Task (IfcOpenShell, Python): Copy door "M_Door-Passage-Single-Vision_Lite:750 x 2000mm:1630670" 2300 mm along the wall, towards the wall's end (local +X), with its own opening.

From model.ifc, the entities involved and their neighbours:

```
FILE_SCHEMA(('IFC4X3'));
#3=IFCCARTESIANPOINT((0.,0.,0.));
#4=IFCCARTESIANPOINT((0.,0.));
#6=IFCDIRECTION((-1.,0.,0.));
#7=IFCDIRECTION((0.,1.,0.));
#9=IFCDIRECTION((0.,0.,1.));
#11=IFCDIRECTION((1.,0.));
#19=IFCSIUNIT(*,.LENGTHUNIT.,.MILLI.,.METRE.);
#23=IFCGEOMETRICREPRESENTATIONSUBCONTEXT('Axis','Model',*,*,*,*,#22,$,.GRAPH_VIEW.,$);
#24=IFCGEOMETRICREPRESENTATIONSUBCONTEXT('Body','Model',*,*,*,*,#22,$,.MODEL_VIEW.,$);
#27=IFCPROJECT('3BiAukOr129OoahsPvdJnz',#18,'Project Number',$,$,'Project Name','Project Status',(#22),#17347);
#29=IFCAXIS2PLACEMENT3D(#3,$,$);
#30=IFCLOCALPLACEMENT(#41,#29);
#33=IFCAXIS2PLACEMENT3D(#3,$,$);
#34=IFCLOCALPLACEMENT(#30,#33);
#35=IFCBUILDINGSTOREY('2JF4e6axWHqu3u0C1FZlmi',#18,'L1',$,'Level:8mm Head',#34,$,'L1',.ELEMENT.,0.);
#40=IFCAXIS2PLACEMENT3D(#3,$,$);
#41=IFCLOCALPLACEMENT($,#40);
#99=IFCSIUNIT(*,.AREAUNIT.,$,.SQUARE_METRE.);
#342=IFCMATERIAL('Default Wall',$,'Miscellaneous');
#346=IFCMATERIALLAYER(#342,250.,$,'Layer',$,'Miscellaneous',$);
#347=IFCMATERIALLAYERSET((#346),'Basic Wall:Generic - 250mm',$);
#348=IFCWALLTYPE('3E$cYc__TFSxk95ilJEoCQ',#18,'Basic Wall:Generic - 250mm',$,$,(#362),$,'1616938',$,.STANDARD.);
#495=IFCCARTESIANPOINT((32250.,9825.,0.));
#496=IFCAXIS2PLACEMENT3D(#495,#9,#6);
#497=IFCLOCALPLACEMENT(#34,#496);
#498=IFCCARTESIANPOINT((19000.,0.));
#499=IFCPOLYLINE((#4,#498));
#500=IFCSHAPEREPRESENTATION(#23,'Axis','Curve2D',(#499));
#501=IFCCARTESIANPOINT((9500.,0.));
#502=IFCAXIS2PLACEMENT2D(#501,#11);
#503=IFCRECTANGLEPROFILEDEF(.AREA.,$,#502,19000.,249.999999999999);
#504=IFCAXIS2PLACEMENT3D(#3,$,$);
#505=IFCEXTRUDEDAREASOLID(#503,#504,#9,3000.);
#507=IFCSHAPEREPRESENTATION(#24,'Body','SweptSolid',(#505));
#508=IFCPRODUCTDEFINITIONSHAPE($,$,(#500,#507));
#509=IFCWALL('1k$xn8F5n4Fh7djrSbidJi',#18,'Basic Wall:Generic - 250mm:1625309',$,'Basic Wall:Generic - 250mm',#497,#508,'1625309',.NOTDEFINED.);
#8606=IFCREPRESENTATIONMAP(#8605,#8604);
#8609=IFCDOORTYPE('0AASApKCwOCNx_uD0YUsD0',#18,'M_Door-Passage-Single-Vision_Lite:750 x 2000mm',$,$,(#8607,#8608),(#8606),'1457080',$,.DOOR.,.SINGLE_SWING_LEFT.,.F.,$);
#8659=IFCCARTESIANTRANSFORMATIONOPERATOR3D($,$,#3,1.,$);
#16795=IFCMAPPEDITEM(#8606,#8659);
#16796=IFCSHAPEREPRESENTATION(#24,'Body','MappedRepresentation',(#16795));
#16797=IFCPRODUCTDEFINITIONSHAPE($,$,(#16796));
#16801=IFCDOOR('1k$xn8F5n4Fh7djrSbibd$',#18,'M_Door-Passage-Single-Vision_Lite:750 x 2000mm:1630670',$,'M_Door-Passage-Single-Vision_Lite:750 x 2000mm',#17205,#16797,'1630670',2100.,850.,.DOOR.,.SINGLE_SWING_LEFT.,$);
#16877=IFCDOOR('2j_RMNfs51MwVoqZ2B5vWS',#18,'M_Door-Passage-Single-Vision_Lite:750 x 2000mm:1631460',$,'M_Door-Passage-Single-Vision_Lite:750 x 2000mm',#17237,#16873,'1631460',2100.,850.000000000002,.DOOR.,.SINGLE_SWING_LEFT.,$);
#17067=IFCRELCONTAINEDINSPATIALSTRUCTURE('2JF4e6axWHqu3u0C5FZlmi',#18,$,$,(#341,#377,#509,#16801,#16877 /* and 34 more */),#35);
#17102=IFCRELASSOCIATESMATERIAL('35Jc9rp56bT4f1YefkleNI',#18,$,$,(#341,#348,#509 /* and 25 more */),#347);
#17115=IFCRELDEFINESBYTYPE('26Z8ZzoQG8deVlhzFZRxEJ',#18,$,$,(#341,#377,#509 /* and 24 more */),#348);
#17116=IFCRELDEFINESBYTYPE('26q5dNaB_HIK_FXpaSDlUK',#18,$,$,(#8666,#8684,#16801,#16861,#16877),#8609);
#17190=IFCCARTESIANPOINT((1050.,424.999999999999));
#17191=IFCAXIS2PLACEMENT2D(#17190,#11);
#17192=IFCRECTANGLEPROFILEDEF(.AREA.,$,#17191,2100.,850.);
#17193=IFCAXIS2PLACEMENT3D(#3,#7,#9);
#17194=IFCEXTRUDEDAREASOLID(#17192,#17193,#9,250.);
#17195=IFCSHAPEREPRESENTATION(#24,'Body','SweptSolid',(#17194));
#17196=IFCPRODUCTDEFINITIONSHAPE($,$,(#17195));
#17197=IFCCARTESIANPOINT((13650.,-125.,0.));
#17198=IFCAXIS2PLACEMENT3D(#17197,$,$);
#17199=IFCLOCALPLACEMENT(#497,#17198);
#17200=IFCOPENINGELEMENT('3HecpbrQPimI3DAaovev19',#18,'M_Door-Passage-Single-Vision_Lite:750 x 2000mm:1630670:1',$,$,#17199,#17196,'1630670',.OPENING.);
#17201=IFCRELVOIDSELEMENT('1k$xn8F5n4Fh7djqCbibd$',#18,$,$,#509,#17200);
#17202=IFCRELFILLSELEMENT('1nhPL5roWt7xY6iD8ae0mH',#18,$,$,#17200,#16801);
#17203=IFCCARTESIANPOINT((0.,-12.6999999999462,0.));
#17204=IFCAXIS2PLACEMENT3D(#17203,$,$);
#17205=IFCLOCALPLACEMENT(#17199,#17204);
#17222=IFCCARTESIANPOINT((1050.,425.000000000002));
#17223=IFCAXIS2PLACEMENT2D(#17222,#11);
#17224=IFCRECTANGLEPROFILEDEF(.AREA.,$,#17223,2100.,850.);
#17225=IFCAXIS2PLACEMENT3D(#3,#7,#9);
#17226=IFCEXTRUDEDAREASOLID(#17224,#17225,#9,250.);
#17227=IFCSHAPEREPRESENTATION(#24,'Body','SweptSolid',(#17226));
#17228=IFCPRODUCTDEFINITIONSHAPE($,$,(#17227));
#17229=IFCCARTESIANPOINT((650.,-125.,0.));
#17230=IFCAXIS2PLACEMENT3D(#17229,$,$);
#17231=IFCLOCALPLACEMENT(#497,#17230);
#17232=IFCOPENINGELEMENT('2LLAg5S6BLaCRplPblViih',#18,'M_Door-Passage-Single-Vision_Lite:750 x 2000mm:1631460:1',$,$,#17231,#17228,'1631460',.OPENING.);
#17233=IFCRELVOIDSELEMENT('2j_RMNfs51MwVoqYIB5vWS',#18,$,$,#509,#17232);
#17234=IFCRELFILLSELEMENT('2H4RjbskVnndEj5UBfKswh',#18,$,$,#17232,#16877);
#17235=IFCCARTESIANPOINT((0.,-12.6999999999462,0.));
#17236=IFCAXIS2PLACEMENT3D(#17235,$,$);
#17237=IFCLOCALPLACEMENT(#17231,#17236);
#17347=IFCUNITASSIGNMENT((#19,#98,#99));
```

```python
import ifcopenshell
import ifcopenshell.api.feature
import ifcopenshell.api.geometry
import ifcopenshell.api.root
import ifcopenshell.geom
import ifcopenshell.util.element
import ifcopenshell.util.placement
import ifcopenshell.util.shape

model = ifcopenshell.open("model.ifc")
settings = ifcopenshell.geom.settings()


def volume(element):
    """Net volume in cubic metres, openings subtracted."""
    shape = ifcopenshell.geom.create_shape(settings, element)
    return ifcopenshell.util.shape.get_volume(shape.geometry)


def reuse_history(source, copy):
    """copy_class also copies each property set's owner history, people and application; keep the originals."""
    for rel in copy.IsDefinedBy:
        if rel.is_a("IfcRelDefinesByProperties") and (history := rel.RelatingPropertyDefinition.OwnerHistory):
            rel.RelatingPropertyDefinition.OwnerHistory = source.OwnerHistory
            ifcopenshell.util.element.remove_deep2(model, history)


door = model.by_guid("1k$xn8F5n4Fh7djrSbibd$")
opening = door.FillsVoids[0].RelatingOpeningElement
wall = opening.VoidsElements[0].RelatingBuildingElement
before = volume(wall)
shift = ifcopenshell.util.placement.get_local_placement(wall.ObjectPlacement)[:3, 0] * 2300.0

# copy_class copies the void relationship, type, container and properties, but no geometry.
new_opening = ifcopenshell.api.root.copy_class(model, product=opening)
new_opening.Representation = ifcopenshell.util.element.copy_deep(
    model, opening.Representation, exclude=["IfcGeometricRepresentationContext", "IfcRepresentationMap"]
)
new_opening.Name = "M_Door-Passage-Single-Vision_Lite:750 x 2000mm"
new_opening.Tag = None
new_door = ifcopenshell.api.root.copy_class(model, product=door)
new_door.Representation = ifcopenshell.util.element.copy_deep(
    model, door.Representation, exclude=["IfcGeometricRepresentationContext", "IfcRepresentationMap"]
)
new_door.Name = "M_Door-Passage-Single-Vision_Lite:750 x 2000mm"
new_door.Tag = None
reuse_history(door, new_door)
ifcopenshell.api.feature.add_filling(model, opening=new_opening, element=new_door)

for old, new in ((opening, new_opening), (door, new_door)):
    matrix = ifcopenshell.util.placement.get_local_placement(old.ObjectPlacement)
    matrix[:3, 3] += shift
    ifcopenshell.api.geometry.edit_object_placement(model, product=new, matrix=matrix, is_si=False)

after = volume(wall)

print(f"wall volume {before:.3f} -> {after:.3f} m3")

model.write("model_updated.ifc")
```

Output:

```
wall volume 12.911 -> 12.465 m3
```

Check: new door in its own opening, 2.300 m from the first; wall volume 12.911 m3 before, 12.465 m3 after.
